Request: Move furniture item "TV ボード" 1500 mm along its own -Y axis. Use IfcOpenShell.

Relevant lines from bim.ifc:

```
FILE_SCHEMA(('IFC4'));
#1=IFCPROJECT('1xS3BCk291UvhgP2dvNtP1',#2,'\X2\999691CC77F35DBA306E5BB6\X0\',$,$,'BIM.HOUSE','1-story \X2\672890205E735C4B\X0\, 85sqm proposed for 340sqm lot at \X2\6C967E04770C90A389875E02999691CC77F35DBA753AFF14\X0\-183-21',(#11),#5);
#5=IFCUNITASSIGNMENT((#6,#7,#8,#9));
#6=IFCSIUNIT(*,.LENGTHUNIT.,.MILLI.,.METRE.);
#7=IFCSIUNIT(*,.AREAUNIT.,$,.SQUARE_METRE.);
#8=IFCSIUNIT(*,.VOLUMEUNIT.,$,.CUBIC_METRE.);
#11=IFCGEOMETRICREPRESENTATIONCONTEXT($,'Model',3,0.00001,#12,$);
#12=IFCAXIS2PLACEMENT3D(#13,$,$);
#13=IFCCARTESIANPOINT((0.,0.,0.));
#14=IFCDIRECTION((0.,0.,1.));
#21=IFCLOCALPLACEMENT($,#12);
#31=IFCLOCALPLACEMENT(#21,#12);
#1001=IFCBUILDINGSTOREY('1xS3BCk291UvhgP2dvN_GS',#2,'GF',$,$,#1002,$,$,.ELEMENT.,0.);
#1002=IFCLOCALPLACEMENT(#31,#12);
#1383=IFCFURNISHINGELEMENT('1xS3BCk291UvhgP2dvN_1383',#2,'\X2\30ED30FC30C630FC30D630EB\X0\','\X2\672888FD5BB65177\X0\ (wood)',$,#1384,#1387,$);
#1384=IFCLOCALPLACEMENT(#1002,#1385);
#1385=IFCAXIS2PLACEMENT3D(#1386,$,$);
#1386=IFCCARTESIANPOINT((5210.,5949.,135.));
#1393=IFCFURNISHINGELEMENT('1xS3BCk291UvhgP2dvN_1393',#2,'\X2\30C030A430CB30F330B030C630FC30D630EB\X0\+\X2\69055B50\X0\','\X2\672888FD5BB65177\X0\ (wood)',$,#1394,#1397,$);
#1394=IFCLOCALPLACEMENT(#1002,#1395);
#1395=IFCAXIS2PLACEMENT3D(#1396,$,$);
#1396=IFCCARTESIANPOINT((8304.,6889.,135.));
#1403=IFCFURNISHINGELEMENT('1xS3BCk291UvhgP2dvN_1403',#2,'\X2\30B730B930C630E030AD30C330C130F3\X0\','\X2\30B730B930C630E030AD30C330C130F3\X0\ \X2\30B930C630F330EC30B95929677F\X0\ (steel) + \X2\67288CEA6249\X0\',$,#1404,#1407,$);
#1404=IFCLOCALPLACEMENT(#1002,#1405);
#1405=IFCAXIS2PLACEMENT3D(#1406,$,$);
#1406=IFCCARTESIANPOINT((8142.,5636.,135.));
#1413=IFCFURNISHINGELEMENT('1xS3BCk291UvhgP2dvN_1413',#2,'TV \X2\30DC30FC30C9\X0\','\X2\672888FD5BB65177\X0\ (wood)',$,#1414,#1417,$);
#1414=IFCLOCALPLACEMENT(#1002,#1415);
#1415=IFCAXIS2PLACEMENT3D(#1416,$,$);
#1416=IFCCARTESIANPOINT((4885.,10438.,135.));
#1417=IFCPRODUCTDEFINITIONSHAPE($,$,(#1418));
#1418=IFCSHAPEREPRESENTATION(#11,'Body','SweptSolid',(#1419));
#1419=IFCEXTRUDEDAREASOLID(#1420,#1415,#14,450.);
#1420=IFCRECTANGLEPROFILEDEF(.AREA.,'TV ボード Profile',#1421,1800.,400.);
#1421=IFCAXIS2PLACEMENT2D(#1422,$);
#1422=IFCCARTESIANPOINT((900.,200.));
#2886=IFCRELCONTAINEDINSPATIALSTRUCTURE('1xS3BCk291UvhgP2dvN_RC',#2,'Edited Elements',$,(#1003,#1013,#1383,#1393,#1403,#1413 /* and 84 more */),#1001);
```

```python
import ifcopenshell
import ifcopenshell.api.geometry
import ifcopenshell.util.placement

model = ifcopenshell.open("bim.ifc")

item = model.by_guid("1xS3BCk291UvhgP2dvN_1413")
matrix = ifcopenshell.util.placement.get_local_placement(item.ObjectPlacement)
matrix[:3, 3] -= matrix[:3, 1] * 1500.0
ifcopenshell.api.geometry.edit_object_placement(model, product=item, matrix=matrix, is_si=False)

print(ifcopenshell.util.placement.get_local_placement(item.ObjectPlacement).round(3) + 0.0)

model.write("bim_edited.ifc")
```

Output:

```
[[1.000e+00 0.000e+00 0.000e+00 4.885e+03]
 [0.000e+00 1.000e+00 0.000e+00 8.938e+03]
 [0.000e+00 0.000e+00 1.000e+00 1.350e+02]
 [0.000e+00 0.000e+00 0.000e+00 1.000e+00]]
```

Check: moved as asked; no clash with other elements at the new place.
